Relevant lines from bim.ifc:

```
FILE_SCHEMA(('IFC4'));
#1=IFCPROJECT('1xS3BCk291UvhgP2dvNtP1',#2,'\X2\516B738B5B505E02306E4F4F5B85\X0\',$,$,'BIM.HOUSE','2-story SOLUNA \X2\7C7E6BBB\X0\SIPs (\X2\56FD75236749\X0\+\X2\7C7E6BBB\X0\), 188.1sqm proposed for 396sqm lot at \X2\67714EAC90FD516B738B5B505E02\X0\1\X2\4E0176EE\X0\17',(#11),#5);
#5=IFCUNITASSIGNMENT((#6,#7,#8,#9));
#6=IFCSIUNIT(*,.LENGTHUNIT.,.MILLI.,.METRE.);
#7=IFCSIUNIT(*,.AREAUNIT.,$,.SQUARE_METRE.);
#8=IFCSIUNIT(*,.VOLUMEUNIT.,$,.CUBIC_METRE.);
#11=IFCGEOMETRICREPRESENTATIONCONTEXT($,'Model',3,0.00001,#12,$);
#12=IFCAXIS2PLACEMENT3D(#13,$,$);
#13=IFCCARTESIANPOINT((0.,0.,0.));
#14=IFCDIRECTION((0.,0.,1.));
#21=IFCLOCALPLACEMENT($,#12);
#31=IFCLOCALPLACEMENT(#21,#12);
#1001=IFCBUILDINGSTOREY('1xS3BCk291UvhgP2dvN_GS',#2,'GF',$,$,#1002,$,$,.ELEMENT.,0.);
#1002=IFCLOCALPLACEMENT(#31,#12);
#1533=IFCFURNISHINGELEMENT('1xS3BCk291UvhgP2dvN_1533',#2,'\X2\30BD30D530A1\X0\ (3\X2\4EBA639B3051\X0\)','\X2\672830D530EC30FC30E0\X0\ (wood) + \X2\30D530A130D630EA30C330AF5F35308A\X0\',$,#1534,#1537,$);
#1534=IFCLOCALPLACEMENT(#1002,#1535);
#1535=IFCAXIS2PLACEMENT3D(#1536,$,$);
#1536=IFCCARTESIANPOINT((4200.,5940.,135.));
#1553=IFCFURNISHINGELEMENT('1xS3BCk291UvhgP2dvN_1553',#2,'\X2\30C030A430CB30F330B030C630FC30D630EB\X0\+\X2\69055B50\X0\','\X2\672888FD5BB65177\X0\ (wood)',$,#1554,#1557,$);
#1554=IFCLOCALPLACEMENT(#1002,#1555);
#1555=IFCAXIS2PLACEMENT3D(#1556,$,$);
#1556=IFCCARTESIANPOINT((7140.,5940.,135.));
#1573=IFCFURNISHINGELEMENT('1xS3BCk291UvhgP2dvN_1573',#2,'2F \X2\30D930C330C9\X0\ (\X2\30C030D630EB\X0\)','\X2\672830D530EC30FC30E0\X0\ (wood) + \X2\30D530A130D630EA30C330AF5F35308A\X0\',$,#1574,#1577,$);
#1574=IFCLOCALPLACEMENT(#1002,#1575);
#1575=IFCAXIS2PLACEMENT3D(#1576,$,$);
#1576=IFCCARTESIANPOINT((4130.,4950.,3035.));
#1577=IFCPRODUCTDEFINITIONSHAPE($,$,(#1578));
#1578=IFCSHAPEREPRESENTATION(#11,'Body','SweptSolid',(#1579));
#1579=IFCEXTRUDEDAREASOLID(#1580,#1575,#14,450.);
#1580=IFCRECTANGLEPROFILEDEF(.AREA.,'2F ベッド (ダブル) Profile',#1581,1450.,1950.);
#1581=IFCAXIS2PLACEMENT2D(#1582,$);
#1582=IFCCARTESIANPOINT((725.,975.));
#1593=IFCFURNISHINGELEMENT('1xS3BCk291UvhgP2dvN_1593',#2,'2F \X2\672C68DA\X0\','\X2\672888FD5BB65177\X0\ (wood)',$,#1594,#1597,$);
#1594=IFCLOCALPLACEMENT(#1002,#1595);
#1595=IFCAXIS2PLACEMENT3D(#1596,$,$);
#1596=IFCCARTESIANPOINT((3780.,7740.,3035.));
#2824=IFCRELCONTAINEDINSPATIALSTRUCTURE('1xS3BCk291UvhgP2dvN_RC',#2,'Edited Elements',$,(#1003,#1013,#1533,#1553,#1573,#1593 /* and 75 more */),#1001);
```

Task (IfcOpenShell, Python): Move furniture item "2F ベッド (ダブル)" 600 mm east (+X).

```python
import ifcopenshell
import ifcopenshell.api.geometry
import ifcopenshell.util.placement

model = ifcopenshell.open("bim.ifc")

item = model.by_guid("1xS3BCk291UvhgP2dvN_1573")
matrix = ifcopenshell.util.placement.get_local_placement(item.ObjectPlacement)
matrix[0, 3] += 600.0
ifcopenshell.api.geometry.edit_object_placement(model, product=item, matrix=matrix, is_si=False)

print(ifcopenshell.util.placement.get_local_placement(item.ObjectPlacement).round(3) + 0.0)

model.write("bim-out.ifc")
```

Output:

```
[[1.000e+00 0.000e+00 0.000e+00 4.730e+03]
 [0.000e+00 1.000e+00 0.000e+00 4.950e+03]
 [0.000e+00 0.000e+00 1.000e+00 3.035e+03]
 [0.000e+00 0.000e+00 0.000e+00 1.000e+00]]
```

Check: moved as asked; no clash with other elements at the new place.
